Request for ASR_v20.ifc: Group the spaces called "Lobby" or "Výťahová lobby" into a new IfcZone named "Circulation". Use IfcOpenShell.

First a look at what the model holds.

```python
import ifcopenshell

model = ifcopenshell.open("ASR_v20.ifc")
print(model.schema)
seen = {}
for space in model.by_type("IfcSpace"):
    seen[space.LongName] = seen.get(space.LongName, 0) + 1
for name, count in sorted(seen.items(), key=str):
    print(count, "x", name)
print("zones:", [z.Name for z in model.by_type("IfcZone")][:20])
```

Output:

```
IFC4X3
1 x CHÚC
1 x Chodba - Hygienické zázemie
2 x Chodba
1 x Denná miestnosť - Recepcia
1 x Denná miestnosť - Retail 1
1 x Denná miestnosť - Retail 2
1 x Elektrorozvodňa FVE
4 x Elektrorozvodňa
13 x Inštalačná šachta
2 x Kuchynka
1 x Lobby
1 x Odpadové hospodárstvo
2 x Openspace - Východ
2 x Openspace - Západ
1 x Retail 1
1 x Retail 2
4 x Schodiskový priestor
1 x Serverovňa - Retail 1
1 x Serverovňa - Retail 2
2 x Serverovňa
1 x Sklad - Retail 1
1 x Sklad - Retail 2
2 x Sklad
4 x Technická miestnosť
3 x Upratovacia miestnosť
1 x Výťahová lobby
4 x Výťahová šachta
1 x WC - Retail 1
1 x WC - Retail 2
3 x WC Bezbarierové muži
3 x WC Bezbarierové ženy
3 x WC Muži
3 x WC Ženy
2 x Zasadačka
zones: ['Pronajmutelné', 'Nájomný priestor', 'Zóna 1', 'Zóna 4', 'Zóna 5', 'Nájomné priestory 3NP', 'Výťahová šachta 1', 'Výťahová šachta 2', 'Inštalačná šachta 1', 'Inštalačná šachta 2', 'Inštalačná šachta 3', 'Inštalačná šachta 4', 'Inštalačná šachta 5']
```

```python
import ifcopenshell
import ifcopenshell.api.group
import ifcopenshell.api.root

model = ifcopenshell.open("ASR_v20.ifc")

names = {"Lobby", "Výťahová lobby"}
spaces = [s for s in model.by_type("IfcSpace") if s.LongName in names]

zone = ifcopenshell.api.root.create_entity(model, ifc_class="IfcZone", name="Circulation")
ifcopenshell.api.group.assign_group(model, products=spaces, group=zone)
print(len(spaces), "spaces in", zone.Name)

model.write("ASR_v20_edited.ifc")
```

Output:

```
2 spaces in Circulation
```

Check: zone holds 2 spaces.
